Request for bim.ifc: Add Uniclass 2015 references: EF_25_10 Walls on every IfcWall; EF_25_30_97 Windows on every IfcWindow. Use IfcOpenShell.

First a look at what the model holds.

```python
import ifcopenshell

model = ifcopenshell.open("bim.ifc")
print(model.schema)
print("classifications:", [c.Name for c in model.by_type("IfcClassification")])
for ifc_class in ("IfcDoor", "IfcRoof", "IfcStair", "IfcWall", "IfcWindow"):
    print(ifc_class, len(model.by_type(ifc_class)))
```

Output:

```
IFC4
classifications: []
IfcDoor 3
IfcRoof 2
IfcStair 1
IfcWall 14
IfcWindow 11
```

```python
import ifcopenshell
import ifcopenshell.api.classification

model = ifcopenshell.open("bim.ifc")

system = ifcopenshell.api.classification.add_classification(model, classification="Uniclass 2015")

codes = {
    "IfcWall": ("EF_25_10", "Walls"),
    "IfcWindow": ("EF_25_30_97", "Windows"),
}
for ifc_class, (code, name) in codes.items():
    products = model.by_type(ifc_class)
    ifcopenshell.api.classification.add_reference(
        model, products=products, classification=system, identification=code, name=name
    )
    print(code, len(products))

model.write("bim_edited.ifc")
```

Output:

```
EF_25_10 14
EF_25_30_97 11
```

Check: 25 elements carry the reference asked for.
